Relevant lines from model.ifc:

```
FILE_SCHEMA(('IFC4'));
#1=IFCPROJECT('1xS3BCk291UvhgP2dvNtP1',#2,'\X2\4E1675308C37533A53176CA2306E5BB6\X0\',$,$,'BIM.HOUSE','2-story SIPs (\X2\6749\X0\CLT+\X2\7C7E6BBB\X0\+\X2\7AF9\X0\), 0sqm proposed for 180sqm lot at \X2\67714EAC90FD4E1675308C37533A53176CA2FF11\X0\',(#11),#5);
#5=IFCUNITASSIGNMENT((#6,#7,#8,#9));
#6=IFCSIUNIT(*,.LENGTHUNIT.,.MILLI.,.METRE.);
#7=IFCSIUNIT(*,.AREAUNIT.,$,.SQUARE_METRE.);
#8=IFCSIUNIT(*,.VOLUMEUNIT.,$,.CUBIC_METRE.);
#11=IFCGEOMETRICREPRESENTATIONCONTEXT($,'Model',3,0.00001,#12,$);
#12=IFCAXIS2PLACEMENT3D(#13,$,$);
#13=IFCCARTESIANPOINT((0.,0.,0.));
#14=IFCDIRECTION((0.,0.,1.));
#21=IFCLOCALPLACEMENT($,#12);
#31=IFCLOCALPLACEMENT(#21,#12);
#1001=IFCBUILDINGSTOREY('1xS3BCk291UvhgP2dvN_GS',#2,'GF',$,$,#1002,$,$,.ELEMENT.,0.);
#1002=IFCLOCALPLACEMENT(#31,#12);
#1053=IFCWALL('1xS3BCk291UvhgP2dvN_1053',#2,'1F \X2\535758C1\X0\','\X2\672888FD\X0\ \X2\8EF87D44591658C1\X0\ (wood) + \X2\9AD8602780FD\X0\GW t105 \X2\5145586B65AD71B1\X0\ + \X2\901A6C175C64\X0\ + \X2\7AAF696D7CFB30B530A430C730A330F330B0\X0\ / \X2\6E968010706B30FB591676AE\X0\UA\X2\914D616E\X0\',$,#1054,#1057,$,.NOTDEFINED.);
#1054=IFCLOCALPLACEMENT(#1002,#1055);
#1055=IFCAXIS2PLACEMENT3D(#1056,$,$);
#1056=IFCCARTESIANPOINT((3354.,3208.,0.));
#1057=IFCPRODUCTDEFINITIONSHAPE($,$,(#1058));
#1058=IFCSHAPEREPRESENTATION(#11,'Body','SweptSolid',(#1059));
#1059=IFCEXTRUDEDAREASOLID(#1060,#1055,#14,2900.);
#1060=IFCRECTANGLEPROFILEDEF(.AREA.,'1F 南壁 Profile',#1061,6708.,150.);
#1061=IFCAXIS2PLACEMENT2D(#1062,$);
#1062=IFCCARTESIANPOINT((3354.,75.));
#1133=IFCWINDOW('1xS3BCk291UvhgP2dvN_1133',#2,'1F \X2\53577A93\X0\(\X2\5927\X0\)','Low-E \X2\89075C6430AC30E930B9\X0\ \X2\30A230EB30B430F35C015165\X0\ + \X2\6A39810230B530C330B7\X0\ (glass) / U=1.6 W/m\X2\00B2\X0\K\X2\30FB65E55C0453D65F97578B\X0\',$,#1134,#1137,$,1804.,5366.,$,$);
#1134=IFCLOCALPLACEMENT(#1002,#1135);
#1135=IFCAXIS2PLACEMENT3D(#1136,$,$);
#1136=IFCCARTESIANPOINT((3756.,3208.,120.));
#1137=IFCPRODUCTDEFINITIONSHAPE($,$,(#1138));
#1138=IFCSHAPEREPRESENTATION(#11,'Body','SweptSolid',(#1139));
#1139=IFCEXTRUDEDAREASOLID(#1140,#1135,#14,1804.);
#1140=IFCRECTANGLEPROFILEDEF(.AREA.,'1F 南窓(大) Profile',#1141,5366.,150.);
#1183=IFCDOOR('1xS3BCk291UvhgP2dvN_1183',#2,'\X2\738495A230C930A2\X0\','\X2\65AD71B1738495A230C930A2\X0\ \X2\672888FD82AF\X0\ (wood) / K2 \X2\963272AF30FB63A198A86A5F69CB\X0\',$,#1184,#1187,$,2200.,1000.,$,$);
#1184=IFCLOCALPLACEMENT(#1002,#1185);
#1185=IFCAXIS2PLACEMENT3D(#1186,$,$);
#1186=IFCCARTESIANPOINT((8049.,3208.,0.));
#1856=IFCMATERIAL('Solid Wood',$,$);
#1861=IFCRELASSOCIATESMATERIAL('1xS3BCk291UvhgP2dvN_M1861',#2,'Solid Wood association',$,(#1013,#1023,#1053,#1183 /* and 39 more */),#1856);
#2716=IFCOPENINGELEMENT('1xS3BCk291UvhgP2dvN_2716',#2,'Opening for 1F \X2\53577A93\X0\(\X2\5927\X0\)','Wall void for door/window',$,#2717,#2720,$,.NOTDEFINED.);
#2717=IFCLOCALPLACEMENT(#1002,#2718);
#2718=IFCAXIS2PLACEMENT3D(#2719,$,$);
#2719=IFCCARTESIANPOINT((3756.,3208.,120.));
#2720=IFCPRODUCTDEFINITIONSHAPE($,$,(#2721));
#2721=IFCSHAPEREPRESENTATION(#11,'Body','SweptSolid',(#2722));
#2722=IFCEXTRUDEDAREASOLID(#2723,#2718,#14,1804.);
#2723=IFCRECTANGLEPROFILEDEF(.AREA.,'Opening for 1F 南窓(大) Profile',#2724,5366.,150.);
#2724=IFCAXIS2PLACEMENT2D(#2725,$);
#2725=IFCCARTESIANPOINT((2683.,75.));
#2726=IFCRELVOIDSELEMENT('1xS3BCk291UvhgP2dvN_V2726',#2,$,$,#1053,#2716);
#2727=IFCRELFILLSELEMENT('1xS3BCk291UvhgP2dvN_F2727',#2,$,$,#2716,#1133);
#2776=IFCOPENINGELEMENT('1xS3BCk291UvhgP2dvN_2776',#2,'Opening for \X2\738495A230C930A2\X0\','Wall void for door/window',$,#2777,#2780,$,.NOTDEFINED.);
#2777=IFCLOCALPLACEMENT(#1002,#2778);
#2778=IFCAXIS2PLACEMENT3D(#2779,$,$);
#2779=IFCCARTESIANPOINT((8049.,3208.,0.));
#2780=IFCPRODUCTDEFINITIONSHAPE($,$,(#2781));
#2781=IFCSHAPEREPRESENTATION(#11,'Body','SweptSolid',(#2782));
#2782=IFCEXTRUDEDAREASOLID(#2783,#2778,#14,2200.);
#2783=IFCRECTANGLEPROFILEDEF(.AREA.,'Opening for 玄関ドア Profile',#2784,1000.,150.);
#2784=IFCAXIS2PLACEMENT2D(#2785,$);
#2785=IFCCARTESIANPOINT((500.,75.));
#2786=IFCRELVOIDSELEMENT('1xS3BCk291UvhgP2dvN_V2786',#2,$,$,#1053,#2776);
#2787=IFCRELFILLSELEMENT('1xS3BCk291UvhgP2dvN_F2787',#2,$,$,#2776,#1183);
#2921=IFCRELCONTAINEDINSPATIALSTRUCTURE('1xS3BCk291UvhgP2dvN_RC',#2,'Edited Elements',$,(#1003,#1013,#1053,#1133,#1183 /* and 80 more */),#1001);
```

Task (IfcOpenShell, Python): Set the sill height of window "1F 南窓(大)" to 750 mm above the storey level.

```python
import numpy as np
import ifcopenshell
import ifcopenshell.api.geometry
import ifcopenshell.geom
import ifcopenshell.util.element
import ifcopenshell.util.placement
import ifcopenshell.util.shape
import ifcopenshell.util.unit

model = ifcopenshell.open("model.ifc")
unit_scale = ifcopenshell.util.unit.calculate_unit_scale(model)

window = model.by_guid("1xS3BCk291UvhgP2dvN_1133")
opening = window.FillsVoids[0].RelatingOpeningElement
storey = ifcopenshell.util.element.get_container(window, ifc_class="IfcBuildingStorey")
level = ifcopenshell.util.placement.get_local_placement(storey.ObjectPlacement)[2, 3]

# The opening's origin need not be at the sill, so measure its lowest point.
shape = ifcopenshell.geom.create_shape(ifcopenshell.geom.settings(), opening)
bottom = ifcopenshell.util.shape.get_shape_bottom_elevation(shape, shape.geometry) / unit_scale
dz = level + 0.75 / unit_scale - bottom

shift = np.array([0.0, 0.0, dz])
# The window is not placed relative to its opening, so move both.
for product in (opening, window):
    matrix = ifcopenshell.util.placement.get_local_placement(product.ObjectPlacement)
    matrix[:3, 3] += shift
    ifcopenshell.api.geometry.edit_object_placement(model, product=product, matrix=matrix, is_si=False)

print(f"moved by {dz * unit_scale:+.3f} m")

model.write("model_edited.ifc")
```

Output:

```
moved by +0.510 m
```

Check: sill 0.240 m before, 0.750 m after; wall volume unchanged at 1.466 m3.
